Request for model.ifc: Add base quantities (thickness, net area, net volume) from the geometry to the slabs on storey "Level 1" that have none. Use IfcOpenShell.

First a look at what the model holds.

```python
import ifcopenshell
import ifcopenshell.util.element
import ifcopenshell.util.unit

model = ifcopenshell.open("model.ifc")
print(model.schema)
for unit_type in ("LENGTHUNIT", "AREAUNIT", "VOLUMEUNIT"):
    print(unit_type, ifcopenshell.util.unit.calculate_unit_scale(model, unit_type))
storey = next(s for s in model.by_type("IfcBuildingStorey") if s.Name == "Level 1")
slabs = [e for e in ifcopenshell.util.element.get_decomposition(storey) if e.is_a("IfcSlab")]
for e in sorted(slabs, key=lambda e: e.id()):
    print(e.id(), e.is_a(), e.Name, list(ifcopenshell.util.element.get_psets(e, qtos_only=True)), sep=" | ")
```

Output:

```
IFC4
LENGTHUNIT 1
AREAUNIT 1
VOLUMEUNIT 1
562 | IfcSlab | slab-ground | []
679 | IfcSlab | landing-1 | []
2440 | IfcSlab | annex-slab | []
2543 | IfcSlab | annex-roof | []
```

```python
import ifcopenshell
import ifcopenshell.api.pset
import ifcopenshell.geom
import ifcopenshell.util.element
import ifcopenshell.util.shape
import ifcopenshell.util.unit

model = ifcopenshell.open("model.ifc")
unit_scale = ifcopenshell.util.unit.calculate_unit_scale(model)
area_scale = ifcopenshell.util.unit.calculate_unit_scale(model, "AREAUNIT")
volume_scale = ifcopenshell.util.unit.calculate_unit_scale(model, "VOLUMEUNIT")
settings = ifcopenshell.geom.settings()

storey = next(s for s in model.by_type("IfcBuildingStorey") if s.Name == "Level 1")
slabs = [e for e in ifcopenshell.util.element.get_decomposition(storey) if e.is_a("IfcSlab")]

for e in sorted(slabs, key=lambda e: e.id()):
    if ifcopenshell.util.element.get_psets(e, qtos_only=True, should_inherit=False):
        continue
    # Geometry comes back in metres, in the element's own axes.
    shape = ifcopenshell.geom.create_shape(settings, e)
    values = {
        "Width": ifcopenshell.util.shape.get_z(shape.geometry) / unit_scale,
        "NetArea": ifcopenshell.util.shape.get_footprint_area(shape.geometry) / area_scale,
        "NetVolume": ifcopenshell.util.shape.get_volume(shape.geometry) / volume_scale,
    }
    qto = ifcopenshell.api.pset.add_qto(model, product=e, name="Qto_SlabBaseQuantities")
    ifcopenshell.api.pset.edit_qto(model, qto=qto, properties=values)
    print(e.id(), {k: round(v, 3) for k, v in values.items()})

model.write("model_edited.ifc")
```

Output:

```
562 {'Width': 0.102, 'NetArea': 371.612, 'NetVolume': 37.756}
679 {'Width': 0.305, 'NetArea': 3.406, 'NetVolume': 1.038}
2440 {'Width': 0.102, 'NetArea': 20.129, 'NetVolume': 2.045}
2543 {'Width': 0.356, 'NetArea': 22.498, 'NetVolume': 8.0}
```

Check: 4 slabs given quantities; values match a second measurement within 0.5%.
